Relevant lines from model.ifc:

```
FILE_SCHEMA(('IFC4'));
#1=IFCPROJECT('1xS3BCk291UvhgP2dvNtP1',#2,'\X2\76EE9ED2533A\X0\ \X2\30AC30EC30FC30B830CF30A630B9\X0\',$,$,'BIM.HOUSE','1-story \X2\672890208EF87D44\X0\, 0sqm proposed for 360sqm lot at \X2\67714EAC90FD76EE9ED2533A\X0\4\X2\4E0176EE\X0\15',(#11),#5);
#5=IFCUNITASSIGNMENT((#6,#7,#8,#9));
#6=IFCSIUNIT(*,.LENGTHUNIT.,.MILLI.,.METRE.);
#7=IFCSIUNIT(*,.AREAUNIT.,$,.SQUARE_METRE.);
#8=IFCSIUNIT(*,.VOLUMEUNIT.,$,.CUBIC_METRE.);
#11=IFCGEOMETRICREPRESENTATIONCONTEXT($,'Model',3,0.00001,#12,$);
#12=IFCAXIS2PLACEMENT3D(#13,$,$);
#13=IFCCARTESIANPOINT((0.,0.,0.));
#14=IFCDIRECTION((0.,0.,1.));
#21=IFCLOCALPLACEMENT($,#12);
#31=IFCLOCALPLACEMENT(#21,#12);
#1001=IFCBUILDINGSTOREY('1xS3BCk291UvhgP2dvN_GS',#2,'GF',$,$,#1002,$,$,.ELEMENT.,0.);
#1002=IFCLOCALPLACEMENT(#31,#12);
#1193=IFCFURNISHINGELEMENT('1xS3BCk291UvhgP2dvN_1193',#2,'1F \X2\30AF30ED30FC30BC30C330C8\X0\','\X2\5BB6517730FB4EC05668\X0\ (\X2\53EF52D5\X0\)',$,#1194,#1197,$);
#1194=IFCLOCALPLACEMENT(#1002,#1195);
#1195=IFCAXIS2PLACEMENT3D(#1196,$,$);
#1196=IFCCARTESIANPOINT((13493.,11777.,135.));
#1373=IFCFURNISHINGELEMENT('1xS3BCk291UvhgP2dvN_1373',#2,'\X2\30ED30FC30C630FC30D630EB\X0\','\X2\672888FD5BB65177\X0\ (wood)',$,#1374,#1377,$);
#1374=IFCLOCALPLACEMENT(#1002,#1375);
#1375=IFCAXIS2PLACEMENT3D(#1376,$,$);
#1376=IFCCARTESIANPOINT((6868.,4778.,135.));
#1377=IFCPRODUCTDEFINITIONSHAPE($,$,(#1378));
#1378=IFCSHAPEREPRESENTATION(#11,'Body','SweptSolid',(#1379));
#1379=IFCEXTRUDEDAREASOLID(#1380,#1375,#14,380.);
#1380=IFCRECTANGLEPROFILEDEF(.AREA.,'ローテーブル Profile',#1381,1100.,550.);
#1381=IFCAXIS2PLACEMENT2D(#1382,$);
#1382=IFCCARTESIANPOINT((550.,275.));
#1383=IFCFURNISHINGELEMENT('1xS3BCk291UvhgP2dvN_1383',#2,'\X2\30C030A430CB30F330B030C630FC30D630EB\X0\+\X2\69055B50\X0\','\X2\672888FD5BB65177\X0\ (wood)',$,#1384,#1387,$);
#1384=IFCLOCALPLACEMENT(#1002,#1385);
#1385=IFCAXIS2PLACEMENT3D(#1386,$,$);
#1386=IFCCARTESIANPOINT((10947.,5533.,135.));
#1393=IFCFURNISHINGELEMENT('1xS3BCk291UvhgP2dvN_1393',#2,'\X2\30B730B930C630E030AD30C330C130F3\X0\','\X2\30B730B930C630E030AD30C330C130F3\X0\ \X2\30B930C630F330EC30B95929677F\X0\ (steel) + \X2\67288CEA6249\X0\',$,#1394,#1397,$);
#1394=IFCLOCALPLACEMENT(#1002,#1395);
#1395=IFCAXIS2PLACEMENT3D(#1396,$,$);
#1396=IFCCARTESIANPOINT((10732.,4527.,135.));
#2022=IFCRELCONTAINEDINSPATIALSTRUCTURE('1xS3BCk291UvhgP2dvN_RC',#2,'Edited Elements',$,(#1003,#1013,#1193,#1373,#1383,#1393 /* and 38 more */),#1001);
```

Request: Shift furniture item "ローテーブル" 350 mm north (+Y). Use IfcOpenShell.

```python
import ifcopenshell
import ifcopenshell.api.geometry
import ifcopenshell.util.placement
import ifcopenshell.util.unit

model = ifcopenshell.open("model.ifc")
unit_scale = ifcopenshell.util.unit.calculate_unit_scale(model)

item = model.by_guid("1xS3BCk291UvhgP2dvN_1373")
matrix = ifcopenshell.util.placement.get_local_placement(item.ObjectPlacement)
matrix[1, 3] += 0.35 / unit_scale
ifcopenshell.api.geometry.edit_object_placement(model, product=item, matrix=matrix, is_si=False)

print(ifcopenshell.util.placement.get_local_placement(item.ObjectPlacement).round(3) + 0.0)

model.write("model-out.ifc")
```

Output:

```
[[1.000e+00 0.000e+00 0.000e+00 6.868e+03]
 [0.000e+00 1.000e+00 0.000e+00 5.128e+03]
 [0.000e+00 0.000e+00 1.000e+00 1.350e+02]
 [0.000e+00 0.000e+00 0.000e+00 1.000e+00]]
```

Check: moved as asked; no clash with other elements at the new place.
